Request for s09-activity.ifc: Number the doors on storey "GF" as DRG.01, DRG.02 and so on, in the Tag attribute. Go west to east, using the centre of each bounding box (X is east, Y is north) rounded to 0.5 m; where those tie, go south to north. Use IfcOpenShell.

First a look at what the model holds.

```python
import ifcopenshell
import ifcopenshell.util.element
import ifcopenshell.util.placement

model = ifcopenshell.open("s09-activity.ifc")
print(model.schema)
storey = next(s for s in model.by_type("IfcBuildingStorey") if s.Name == "GF")
doors = [e for e in ifcopenshell.util.element.get_decomposition(storey) if e.is_a("IfcDoor")]
for e in sorted(doors, key=lambda e: e.id()):
    origin = ifcopenshell.util.placement.get_local_placement(e.ObjectPlacement)[:3, 3]
    print(e.id(), e.Tag, e.Name, origin.round(2) + 0.0, sep=" | ")
```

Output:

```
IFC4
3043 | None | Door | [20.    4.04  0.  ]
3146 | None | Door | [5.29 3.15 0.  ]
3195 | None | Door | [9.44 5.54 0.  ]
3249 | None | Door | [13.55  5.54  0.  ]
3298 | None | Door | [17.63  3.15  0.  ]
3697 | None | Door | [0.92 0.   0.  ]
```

```python
import ifcopenshell
import ifcopenshell.geom
import ifcopenshell.util.element
import ifcopenshell.util.shape

model = ifcopenshell.open("s09-activity.ifc")
settings = ifcopenshell.geom.settings()
settings.set("use-world-coords", True)


def centre(element):
    shape = ifcopenshell.geom.create_shape(settings, element)
    return ifcopenshell.util.shape.get_bbox_centroid(shape.geometry)


storey = next(s for s in model.by_type("IfcBuildingStorey") if s.Name == "GF")
doors = [e for e in ifcopenshell.util.element.get_decomposition(storey) if e.is_a("IfcDoor")]

# Insertion points can sit at a corner or the storey origin, so sort by the geometry (in metres).
centres = {e: centre(e) for e in doors}
doors.sort(key=lambda e: (round(centres[e][0] / 0.5), centres[e][1]))

for i, e in enumerate(doors, start=1):
    number = f"DRG.{i:02d}"
    e.Tag = number
    print(e.id(), number)

model.write("s09-activity_v2.ifc")
```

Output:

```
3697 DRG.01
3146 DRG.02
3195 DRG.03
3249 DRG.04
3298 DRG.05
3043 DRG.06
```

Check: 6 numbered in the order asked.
